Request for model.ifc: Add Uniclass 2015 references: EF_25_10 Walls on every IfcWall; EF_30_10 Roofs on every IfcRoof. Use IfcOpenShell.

First a look at what the model holds.

```python
import ifcopenshell

model = ifcopenshell.open("model.ifc")
print(model.schema)
print("classifications:", [c.Name for c in model.by_type("IfcClassification")])
for ifc_class in ("IfcDoor", "IfcRoof", "IfcStair", "IfcWall", "IfcWindow"):
    print(ifc_class, len(model.by_type(ifc_class)))
```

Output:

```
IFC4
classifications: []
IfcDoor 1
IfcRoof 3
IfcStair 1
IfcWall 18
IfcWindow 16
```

```python
import ifcopenshell
import ifcopenshell.api.classification

model = ifcopenshell.open("model.ifc")

system = ifcopenshell.api.classification.add_classification(model, classification="Uniclass 2015")

codes = {
    "IfcWall": ("EF_25_10", "Walls"),
    "IfcRoof": ("EF_30_10", "Roofs"),
}
for ifc_class, (code, name) in codes.items():
    products = model.by_type(ifc_class)
    ifcopenshell.api.classification.add_reference(
        model, products=products, classification=system, identification=code, name=name
    )
    print(code, len(products))

model.write("model_v2.ifc")
```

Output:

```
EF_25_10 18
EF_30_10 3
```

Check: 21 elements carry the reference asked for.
